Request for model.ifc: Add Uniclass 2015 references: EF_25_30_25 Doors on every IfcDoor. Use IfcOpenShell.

First a look at what the model holds.

```python
import ifcopenshell

model = ifcopenshell.open("model.ifc")
print(model.schema)
print("classifications:", [c.Name for c in model.by_type("IfcClassification")])
for ifc_class in ("IfcDoor", "IfcRoof", "IfcStair", "IfcWall", "IfcWindow"):
    print(ifc_class, len(model.by_type(ifc_class)))
```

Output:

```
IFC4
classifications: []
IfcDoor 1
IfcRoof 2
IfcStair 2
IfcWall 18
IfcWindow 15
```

```python
import ifcopenshell
import ifcopenshell.api.classification

model = ifcopenshell.open("model.ifc")

system = ifcopenshell.api.classification.add_classification(model, classification="Uniclass 2015")

codes = {
    "IfcDoor": ("EF_25_30_25", "Doors"),
}
for ifc_class, (code, name) in codes.items():
    products = model.by_type(ifc_class)
    ifcopenshell.api.classification.add_reference(
        model, products=products, classification=system, identification=code, name=name
    )
    print(code, len(products))

model.write("model_updated.ifc")
```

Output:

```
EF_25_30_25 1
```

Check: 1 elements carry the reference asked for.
